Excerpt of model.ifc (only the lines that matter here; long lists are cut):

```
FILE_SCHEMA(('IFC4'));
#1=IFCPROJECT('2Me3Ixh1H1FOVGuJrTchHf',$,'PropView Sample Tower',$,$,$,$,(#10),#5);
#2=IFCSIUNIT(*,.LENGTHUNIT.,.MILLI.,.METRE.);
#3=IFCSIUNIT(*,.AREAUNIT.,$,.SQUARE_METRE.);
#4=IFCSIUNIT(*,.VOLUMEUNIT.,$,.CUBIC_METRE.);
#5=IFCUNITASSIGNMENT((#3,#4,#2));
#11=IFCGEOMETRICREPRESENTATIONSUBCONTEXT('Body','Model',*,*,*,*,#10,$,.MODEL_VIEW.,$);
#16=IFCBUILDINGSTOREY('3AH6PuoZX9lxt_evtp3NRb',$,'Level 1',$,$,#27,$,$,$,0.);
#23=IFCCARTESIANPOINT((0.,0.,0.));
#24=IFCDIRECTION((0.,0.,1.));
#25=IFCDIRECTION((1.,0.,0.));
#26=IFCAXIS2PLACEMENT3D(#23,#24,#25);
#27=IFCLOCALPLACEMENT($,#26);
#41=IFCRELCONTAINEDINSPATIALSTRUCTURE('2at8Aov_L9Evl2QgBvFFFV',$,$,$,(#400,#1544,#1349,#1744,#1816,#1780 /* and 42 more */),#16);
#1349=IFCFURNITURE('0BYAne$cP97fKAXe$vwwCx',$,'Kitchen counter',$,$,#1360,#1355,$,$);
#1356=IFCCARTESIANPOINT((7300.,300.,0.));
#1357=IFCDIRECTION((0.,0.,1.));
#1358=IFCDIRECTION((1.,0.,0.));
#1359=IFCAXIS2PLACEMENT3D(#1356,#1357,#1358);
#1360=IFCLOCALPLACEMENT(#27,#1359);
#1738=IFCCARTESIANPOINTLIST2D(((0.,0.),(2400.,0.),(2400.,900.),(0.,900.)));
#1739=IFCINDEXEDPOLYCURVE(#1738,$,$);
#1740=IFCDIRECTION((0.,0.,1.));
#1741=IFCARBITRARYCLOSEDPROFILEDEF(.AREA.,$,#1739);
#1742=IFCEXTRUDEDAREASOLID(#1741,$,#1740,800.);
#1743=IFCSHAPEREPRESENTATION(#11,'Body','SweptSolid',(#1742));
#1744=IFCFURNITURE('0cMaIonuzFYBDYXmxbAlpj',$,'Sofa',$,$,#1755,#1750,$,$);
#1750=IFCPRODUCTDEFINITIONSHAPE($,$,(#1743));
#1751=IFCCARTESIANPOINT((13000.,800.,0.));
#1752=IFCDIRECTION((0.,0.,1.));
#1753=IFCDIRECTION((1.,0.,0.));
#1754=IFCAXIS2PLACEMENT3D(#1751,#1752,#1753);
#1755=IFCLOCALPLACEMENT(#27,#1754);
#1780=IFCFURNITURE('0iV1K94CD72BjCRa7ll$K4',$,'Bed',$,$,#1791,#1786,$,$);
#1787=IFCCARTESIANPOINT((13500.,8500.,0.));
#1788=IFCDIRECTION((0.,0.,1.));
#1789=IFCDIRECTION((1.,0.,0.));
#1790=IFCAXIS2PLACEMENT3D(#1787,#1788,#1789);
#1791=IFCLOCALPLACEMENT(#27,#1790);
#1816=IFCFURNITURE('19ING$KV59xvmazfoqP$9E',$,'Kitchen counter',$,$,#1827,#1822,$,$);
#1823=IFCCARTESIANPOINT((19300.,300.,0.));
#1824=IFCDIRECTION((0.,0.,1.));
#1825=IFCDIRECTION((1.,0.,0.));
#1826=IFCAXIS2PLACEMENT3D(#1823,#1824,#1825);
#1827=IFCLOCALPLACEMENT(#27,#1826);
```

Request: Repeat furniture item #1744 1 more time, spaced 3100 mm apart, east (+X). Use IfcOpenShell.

```python
import numpy as np
import ifcopenshell
import ifcopenshell.api.geometry
import ifcopenshell.api.root
import ifcopenshell.util.element
import ifcopenshell.util.placement

model = ifcopenshell.open("model.ifc")

source = model.by_guid("0cMaIonuzFYBDYXmxbAlpj")
base = ifcopenshell.util.placement.get_local_placement(source.ObjectPlacement)
step = np.array([1.0, 0.0, 0.0]) * 3100.0

for i in range(1, 2):
    copy = ifcopenshell.api.root.copy_class(model, product=source)
    copy.Representation = ifcopenshell.util.element.copy_deep(
        model, source.Representation, exclude=["IfcGeometricRepresentationContext", "IfcRepresentationMap"]
    )
    matrix = base.copy()
    matrix[:3, 3] += i * step
    print("added at", matrix[:3, 3].round(3) + 0.0)
    ifcopenshell.api.geometry.edit_object_placement(model, product=copy, matrix=matrix, is_si=False)

model.write("model_updated.ifc")
```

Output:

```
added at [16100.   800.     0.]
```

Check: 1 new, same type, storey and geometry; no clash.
